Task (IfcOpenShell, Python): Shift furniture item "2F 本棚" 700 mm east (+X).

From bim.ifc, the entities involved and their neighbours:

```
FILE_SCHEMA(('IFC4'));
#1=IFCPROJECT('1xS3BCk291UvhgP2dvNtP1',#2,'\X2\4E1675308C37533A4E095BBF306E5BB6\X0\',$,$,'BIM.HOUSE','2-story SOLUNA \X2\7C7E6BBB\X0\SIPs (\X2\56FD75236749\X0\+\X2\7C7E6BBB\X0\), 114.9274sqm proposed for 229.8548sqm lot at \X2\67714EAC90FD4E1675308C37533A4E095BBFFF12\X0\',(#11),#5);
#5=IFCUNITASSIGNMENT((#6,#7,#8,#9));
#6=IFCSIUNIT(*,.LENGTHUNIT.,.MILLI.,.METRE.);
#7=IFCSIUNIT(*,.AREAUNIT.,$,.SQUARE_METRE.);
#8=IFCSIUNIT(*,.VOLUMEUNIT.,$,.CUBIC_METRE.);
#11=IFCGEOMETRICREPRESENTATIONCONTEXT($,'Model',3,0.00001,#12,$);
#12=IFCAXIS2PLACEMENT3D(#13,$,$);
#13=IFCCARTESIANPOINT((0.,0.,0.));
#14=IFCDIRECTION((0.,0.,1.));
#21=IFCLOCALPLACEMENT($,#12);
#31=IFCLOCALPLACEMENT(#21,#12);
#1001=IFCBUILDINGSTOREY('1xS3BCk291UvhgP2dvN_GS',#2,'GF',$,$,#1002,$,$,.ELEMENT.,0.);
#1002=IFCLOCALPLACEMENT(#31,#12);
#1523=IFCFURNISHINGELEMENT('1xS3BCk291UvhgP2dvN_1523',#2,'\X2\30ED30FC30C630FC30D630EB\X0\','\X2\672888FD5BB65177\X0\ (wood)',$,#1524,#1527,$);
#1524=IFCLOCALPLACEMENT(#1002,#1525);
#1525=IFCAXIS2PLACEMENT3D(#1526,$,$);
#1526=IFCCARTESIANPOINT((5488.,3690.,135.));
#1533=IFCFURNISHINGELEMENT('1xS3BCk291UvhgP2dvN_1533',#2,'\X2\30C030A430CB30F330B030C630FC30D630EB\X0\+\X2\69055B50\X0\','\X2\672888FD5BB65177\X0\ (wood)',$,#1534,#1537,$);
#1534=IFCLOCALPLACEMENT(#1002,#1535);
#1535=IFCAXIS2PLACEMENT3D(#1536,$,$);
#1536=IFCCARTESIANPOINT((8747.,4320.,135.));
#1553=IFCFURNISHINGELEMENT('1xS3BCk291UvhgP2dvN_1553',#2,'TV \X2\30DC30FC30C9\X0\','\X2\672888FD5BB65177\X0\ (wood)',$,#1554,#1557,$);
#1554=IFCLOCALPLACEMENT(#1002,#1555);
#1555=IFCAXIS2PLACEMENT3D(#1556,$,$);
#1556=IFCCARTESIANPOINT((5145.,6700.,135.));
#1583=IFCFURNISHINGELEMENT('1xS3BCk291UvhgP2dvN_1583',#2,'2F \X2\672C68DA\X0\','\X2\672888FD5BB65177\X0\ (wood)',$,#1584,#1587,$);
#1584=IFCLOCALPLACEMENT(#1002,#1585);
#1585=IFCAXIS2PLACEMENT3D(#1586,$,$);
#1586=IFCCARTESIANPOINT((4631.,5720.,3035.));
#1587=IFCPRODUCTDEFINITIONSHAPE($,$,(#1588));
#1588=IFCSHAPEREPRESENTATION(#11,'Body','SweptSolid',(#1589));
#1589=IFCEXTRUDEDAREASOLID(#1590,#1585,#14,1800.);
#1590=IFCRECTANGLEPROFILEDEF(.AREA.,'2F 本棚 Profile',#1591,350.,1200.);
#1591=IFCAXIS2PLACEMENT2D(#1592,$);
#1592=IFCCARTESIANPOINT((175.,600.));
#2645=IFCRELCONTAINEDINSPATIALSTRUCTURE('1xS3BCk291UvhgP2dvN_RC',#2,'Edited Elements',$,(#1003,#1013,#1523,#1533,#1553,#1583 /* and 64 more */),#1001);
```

```python
import ifcopenshell
import ifcopenshell.api.geometry
import ifcopenshell.util.placement

model = ifcopenshell.open("bim.ifc")

item = model.by_guid("1xS3BCk291UvhgP2dvN_1583")
matrix = ifcopenshell.util.placement.get_local_placement(item.ObjectPlacement)
matrix[0, 3] += 700.0
ifcopenshell.api.geometry.edit_object_placement(model, product=item, matrix=matrix, is_si=False)

print(ifcopenshell.util.placement.get_local_placement(item.ObjectPlacement).round(3) + 0.0)

model.write("bim_updated.ifc")
```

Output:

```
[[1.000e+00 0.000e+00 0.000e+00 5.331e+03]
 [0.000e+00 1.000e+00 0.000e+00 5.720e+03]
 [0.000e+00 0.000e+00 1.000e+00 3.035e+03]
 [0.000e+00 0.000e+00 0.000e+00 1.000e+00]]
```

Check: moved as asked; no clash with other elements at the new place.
